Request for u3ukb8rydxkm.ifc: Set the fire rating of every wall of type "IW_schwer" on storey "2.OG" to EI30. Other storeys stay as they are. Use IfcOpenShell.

First a look at what the model holds.

```python
import ifcopenshell
import ifcopenshell.util.element

model = ifcopenshell.open("u3ukb8rydxkm.ifc")
print(model.schema)
storey = next(s for s in model.by_type("IfcBuildingStorey") if s.Name == "2.OG")
walls = [e for e in ifcopenshell.util.element.get_decomposition(storey) if e.is_a("IfcWall")]
seen = {}
for e in walls:
    element_type = ifcopenshell.util.element.get_type(e)
    key = (element_type.Name if element_type != e and element_type else None, ifcopenshell.util.element.get_pset(e, "Pset_WallCommon", "FireRating"))
    seen[key] = seen.get(key, 0) + 1
for (name, value), count in sorted(seen.items(), key=str):
    print(count, "x", name, "|", value)
```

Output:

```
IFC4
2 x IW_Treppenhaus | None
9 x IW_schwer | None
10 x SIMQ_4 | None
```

```python
import ifcopenshell
import ifcopenshell.api.pset
import ifcopenshell.util.element

model = ifcopenshell.open("u3ukb8rydxkm.ifc")

storey = next(s for s in model.by_type("IfcBuildingStorey") if s.Name == "2.OG")
walls = [e for e in ifcopenshell.util.element.get_decomposition(storey) if e.is_a("IfcWall")]

count = 0
for e in walls:
    element_type = ifcopenshell.util.element.get_type(e)
    if element_type in (None, e) or element_type.Name != "IW_schwer":
        continue
    # add_pset returns the element's existing set when there is one.
    pset = ifcopenshell.api.pset.add_pset(model, product=e, name="Pset_WallCommon")
    ifcopenshell.api.pset.edit_pset(model, pset=pset, properties={"FireRating": "EI30"})
    count += 1

print(count, "walls updated")

model.write("u3ukb8rydxkm_v2.ifc")
```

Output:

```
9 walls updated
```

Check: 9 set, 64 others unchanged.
